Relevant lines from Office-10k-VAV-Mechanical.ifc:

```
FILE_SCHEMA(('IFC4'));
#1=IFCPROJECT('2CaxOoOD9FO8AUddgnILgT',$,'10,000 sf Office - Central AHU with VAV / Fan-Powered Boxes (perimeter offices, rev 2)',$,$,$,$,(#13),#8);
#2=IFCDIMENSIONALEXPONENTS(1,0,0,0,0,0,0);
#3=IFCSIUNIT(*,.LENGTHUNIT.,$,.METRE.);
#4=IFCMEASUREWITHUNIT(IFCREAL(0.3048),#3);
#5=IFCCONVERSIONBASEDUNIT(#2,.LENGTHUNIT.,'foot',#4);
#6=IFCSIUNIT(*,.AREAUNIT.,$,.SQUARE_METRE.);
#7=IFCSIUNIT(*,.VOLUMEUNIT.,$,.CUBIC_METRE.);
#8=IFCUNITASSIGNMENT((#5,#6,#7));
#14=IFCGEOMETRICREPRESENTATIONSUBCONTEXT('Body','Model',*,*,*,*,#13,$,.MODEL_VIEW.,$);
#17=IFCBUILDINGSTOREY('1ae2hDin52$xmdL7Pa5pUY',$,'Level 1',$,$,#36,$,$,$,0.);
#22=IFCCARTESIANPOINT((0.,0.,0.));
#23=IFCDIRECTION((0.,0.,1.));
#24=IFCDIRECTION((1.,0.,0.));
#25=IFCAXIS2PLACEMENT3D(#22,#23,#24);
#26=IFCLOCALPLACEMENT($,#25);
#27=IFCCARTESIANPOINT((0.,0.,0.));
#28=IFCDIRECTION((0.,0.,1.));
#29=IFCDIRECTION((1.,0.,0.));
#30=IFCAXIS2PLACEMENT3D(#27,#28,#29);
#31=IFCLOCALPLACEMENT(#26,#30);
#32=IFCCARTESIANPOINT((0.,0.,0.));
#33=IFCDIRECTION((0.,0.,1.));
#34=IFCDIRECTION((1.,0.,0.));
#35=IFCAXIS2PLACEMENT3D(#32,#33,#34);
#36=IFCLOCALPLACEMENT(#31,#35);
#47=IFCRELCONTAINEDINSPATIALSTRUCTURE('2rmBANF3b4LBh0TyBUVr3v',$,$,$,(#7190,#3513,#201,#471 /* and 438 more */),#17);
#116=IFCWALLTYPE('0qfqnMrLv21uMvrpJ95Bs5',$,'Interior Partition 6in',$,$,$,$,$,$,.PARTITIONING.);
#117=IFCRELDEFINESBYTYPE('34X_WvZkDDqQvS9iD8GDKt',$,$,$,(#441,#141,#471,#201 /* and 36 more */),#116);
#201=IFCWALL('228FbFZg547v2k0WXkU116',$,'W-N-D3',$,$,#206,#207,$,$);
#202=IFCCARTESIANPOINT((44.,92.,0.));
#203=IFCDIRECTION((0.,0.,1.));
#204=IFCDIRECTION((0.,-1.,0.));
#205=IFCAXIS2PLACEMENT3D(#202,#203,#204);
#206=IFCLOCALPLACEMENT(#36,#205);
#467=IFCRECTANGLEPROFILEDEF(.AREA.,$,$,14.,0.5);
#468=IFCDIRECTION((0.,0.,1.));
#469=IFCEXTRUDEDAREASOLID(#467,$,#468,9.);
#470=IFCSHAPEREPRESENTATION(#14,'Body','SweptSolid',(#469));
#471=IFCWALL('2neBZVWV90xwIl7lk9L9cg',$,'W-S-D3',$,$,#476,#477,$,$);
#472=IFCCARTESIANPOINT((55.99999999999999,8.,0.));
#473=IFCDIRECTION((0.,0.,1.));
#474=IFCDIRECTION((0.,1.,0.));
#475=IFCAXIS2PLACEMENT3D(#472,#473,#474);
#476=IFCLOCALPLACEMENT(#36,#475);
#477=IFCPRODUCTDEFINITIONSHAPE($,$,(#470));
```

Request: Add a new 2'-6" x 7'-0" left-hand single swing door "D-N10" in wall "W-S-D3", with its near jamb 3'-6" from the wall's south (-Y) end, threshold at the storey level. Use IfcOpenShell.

```python
import numpy as np
import ifcopenshell
import ifcopenshell.api.feature
import ifcopenshell.api.geometry
import ifcopenshell.api.root
import ifcopenshell.api.spatial
import ifcopenshell.geom
import ifcopenshell.util.element
import ifcopenshell.util.placement
import ifcopenshell.util.representation
import ifcopenshell.util.shape
import ifcopenshell.util.unit

model = ifcopenshell.open("Office-10k-VAV-Mechanical.ifc")
unit_scale = ifcopenshell.util.unit.calculate_unit_scale(model)
settings = ifcopenshell.geom.settings()


def volume(element):
    """Net volume in cubic metres, openings subtracted."""
    shape = ifcopenshell.geom.create_shape(settings, element)
    return ifcopenshell.util.shape.get_volume(shape.geometry)


wall = model.by_id(471)
storey = ifcopenshell.util.element.get_container(wall, ifc_class="IfcBuildingStorey")
context = ifcopenshell.util.representation.get_context(model, "Model", "Body", "MODEL_VIEW")
before = volume(wall)

width, height, from_end, sill = 0.762, 2.1336, 1.0668, 0.0  # metres

# The wall runs along its own X axis, and the end named is its -X end.
wall_shape = ifcopenshell.geom.create_shape(settings, wall)
x, y, z = ifcopenshell.util.shape.get_vertices(wall_shape.geometry).T
start = x.min() + from_end
face, thickness = float(y.min()), float(y.max() - y.min())
wall_matrix = ifcopenshell.util.placement.get_local_placement(wall.ObjectPlacement)
level = ifcopenshell.util.placement.get_local_placement(storey.ObjectPlacement)[2, 3]


def in_wall(x, y):
    """Placement at x, y metres in the wall's axes, at sill height."""
    matrix = wall_matrix.copy()
    matrix[:, 3] = wall_matrix @ np.array([x / unit_scale, y / unit_scale, 0.0, 1.0])
    matrix[2, 3] = level + sill / unit_scale
    return matrix


# Opening: a box that overshoots both wall faces by 50 mm.
opening = ifcopenshell.api.root.create_entity(model, ifc_class="IfcOpeningElement", predefined_type="OPENING")
box = ifcopenshell.api.geometry.add_wall_representation(
    model, context=context, length=width, height=height, thickness=thickness + 0.1
)
ifcopenshell.api.geometry.assign_representation(model, product=opening, representation=box)
ifcopenshell.api.geometry.edit_object_placement(model, product=opening, matrix=in_wall(start, face - 0.05), is_si=False)
ifcopenshell.api.feature.add_feature(model, feature=opening, element=wall)

door = ifcopenshell.api.root.create_entity(model, ifc_class="IfcDoor", name="D-N10", predefined_type="DOOR")
door.OverallWidth, door.OverallHeight = width / unit_scale, height / unit_scale
door.OperationType = "SINGLE_SWING_LEFT"
body = ifcopenshell.api.geometry.add_door_representation(
    model,
    context=context,
    overall_width=door.OverallWidth,
    overall_height=door.OverallHeight,
    operation_type="SINGLE_SWING_LEFT",
    lining_properties={"LiningDepth": thickness / unit_scale, "ThresholdDepth": thickness / unit_scale},
)
ifcopenshell.api.geometry.assign_representation(model, product=door, representation=body)
ifcopenshell.api.spatial.assign_container(model, products=[door], relating_structure=storey)
ifcopenshell.api.feature.add_filling(model, opening=opening, element=door)

# The lining spans the wall, so the door starts at the wall face.
ifcopenshell.api.geometry.edit_object_placement(model, product=door, matrix=in_wall(start, face), is_si=False)

after = volume(wall)

print(f"wall volume {before:.3f} -> {after:.3f} m3")

model.write("Office-10k-VAV-Mechanical_v2.ifc")
```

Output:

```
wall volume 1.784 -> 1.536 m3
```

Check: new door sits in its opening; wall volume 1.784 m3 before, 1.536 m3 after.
